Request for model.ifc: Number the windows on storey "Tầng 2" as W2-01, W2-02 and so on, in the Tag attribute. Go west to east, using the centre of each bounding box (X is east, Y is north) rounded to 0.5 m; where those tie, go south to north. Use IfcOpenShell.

First a look at what the model holds.

```python
import ifcopenshell
import ifcopenshell.util.element
import ifcopenshell.util.placement

model = ifcopenshell.open("model.ifc")
print(model.schema)
storey = next(s for s in model.by_type("IfcBuildingStorey") if s.Name == "Tầng 2")
windows = [e for e in ifcopenshell.util.element.get_decomposition(storey) if e.is_a("IfcWindow")]
for e in sorted(windows, key=lambda e: e.id()):
    origin = ifcopenshell.util.placement.get_local_placement(e.ObjectPlacement)[:3, 3]
    print(e.id(), e.Tag, e.Name, origin.round(2) + 0.0, sep=" | ")
```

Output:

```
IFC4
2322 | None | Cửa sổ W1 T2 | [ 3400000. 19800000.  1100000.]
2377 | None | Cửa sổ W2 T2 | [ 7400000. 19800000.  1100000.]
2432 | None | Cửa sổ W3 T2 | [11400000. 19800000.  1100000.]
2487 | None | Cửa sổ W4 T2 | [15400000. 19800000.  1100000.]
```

```python
import ifcopenshell
import ifcopenshell.geom
import ifcopenshell.util.element
import ifcopenshell.util.shape

model = ifcopenshell.open("model.ifc")
settings = ifcopenshell.geom.settings()
settings.set("use-world-coords", True)


def centre(element):
    shape = ifcopenshell.geom.create_shape(settings, element)
    return ifcopenshell.util.shape.get_bbox_centroid(shape.geometry)


storey = next(s for s in model.by_type("IfcBuildingStorey") if s.Name == "Tầng 2")
windows = [e for e in ifcopenshell.util.element.get_decomposition(storey) if e.is_a("IfcWindow")]

# Insertion points can sit at a corner or the storey origin, so sort by the geometry (in metres).
centres = {e: centre(e) for e in windows}
windows.sort(key=lambda e: (round(centres[e][0] / 0.5), centres[e][1]))

for i, e in enumerate(windows, start=1):
    number = f"W2-{i:02d}"
    e.Tag = number
    print(e.id(), number)

model.write("model_updated.ifc")
```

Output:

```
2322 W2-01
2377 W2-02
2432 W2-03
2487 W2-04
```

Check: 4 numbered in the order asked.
